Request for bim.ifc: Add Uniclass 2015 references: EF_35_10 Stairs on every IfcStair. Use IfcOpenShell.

First a look at what the model holds.

```python
import ifcopenshell

model = ifcopenshell.open("bim.ifc")
print(model.schema)
print("classifications:", [c.Name for c in model.by_type("IfcClassification")])
for ifc_class in ("IfcDoor", "IfcRoof", "IfcStair", "IfcWall", "IfcWindow"):
    print(ifc_class, len(model.by_type(ifc_class)))
```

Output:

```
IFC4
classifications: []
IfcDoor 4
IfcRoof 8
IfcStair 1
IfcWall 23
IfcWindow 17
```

```python
import ifcopenshell
import ifcopenshell.api.classification

model = ifcopenshell.open("bim.ifc")

system = ifcopenshell.api.classification.add_classification(model, classification="Uniclass 2015")

codes = {
    "IfcStair": ("EF_35_10", "Stairs"),
}
for ifc_class, (code, name) in codes.items():
    products = model.by_type(ifc_class)
    ifcopenshell.api.classification.add_reference(
        model, products=products, classification=system, identification=code, name=name
    )
    print(code, len(products))

model.write("bim_rev.ifc")
```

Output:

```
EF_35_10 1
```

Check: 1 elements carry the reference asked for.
